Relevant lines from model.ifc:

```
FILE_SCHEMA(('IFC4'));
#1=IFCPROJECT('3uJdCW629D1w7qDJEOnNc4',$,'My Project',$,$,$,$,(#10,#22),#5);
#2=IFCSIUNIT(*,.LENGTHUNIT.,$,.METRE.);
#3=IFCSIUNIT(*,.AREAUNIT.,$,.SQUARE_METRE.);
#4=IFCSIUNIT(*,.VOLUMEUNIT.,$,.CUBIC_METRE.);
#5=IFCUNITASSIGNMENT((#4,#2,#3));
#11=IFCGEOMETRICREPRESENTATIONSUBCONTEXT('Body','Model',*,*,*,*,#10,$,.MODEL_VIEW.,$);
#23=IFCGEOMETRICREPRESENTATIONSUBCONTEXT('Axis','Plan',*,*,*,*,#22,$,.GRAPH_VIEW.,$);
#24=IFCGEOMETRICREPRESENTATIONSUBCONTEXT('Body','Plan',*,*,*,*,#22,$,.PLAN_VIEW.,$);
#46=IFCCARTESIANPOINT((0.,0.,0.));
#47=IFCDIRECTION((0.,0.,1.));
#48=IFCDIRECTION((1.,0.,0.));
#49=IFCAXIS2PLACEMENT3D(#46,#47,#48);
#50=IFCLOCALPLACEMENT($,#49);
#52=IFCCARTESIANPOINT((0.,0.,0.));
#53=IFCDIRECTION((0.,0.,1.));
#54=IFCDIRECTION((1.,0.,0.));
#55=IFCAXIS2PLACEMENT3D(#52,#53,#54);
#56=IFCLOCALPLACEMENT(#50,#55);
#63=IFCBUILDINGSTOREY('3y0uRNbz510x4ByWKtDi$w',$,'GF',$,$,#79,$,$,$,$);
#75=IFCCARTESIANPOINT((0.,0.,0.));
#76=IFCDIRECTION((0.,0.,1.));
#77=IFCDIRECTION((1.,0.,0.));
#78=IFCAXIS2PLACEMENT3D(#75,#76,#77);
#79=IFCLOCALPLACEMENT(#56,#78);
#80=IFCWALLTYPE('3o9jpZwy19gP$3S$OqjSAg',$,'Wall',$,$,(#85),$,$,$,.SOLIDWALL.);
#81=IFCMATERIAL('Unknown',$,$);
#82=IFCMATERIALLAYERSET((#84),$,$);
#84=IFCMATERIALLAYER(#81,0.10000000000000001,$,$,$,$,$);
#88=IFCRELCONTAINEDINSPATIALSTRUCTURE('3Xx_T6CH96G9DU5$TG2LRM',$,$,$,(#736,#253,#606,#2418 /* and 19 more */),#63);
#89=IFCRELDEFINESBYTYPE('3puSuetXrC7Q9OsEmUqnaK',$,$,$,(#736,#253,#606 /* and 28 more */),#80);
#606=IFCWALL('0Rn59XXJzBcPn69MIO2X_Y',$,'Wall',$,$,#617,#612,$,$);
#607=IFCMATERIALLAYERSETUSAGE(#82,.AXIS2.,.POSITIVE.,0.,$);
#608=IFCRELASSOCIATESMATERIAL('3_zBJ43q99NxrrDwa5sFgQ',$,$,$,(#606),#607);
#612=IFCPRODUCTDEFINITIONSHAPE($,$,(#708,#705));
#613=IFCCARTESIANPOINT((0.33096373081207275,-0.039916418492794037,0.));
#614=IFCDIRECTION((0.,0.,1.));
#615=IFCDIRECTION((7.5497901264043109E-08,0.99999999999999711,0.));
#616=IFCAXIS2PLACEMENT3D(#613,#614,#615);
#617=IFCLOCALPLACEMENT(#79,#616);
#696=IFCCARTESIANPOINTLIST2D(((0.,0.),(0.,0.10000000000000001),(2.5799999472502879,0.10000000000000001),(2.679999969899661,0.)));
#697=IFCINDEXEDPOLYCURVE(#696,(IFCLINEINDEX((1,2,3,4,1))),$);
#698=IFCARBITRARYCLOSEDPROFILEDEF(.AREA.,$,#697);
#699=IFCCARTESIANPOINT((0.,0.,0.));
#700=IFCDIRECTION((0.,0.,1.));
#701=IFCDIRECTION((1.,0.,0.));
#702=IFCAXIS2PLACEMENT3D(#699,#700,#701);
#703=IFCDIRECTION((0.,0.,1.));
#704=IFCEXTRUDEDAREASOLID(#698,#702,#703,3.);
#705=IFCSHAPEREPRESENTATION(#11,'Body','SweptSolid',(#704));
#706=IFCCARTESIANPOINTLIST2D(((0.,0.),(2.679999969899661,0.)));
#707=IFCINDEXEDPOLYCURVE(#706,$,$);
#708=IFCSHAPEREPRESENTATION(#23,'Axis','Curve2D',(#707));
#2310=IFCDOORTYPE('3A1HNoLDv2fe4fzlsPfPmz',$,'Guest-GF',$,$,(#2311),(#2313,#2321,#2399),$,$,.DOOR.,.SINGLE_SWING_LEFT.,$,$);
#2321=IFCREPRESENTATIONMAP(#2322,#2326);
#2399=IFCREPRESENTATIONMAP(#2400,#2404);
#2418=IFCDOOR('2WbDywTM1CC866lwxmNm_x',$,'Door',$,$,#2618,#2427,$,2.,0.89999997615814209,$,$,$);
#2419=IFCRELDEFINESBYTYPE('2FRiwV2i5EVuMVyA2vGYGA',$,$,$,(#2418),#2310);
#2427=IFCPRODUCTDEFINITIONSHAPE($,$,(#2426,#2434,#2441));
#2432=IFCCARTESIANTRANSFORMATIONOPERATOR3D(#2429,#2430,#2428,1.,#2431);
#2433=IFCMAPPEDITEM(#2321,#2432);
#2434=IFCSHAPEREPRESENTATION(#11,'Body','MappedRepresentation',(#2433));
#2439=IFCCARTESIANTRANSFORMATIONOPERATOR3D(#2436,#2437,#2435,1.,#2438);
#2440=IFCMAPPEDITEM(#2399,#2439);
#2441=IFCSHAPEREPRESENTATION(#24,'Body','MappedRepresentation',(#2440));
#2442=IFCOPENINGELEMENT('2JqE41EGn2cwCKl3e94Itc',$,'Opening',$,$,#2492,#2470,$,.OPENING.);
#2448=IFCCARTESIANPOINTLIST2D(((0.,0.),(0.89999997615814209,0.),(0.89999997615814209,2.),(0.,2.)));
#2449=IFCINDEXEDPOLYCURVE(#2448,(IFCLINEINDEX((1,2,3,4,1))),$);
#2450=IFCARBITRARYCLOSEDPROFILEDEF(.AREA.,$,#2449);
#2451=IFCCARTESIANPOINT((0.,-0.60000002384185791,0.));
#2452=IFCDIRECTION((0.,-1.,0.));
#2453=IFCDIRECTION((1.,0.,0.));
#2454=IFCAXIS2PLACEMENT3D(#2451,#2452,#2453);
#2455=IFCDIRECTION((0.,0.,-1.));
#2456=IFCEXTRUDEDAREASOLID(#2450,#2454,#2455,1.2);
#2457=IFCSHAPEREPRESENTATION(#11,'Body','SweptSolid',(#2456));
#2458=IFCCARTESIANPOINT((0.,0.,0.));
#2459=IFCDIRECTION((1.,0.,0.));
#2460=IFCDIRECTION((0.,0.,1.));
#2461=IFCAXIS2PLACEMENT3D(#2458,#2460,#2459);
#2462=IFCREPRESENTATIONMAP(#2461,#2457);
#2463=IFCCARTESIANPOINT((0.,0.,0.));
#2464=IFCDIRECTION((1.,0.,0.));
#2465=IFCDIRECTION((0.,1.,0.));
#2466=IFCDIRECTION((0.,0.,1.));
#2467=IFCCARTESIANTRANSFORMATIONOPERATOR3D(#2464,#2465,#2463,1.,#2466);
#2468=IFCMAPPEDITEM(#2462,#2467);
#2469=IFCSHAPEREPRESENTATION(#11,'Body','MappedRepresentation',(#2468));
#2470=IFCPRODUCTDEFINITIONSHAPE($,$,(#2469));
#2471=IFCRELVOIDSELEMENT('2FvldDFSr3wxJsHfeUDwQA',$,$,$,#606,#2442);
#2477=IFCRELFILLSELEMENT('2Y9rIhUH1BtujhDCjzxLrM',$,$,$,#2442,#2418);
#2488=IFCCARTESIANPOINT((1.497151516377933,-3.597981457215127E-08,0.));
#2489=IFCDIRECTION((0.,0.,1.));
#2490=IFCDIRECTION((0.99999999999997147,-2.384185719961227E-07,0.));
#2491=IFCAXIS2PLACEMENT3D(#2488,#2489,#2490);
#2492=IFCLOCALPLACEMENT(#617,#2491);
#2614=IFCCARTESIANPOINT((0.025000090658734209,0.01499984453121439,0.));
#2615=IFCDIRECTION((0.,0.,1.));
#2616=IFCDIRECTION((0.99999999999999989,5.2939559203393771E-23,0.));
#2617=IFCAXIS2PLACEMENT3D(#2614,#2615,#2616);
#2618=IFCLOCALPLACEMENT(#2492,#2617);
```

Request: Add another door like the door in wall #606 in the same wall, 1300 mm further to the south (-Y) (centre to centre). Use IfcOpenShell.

```python
import ifcopenshell
import ifcopenshell.api.feature
import ifcopenshell.api.geometry
import ifcopenshell.api.root
import ifcopenshell.geom
import ifcopenshell.util.element
import ifcopenshell.util.placement
import ifcopenshell.util.shape

model = ifcopenshell.open("model.ifc")
settings = ifcopenshell.geom.settings()


def volume(element):
    """Net volume in cubic metres, openings subtracted."""
    shape = ifcopenshell.geom.create_shape(settings, element)
    return ifcopenshell.util.shape.get_volume(shape.geometry)


door = model.by_guid("2WbDywTM1CC866lwxmNm_x")
opening = door.FillsVoids[0].RelatingOpeningElement
wall = opening.VoidsElements[0].RelatingBuildingElement
before = volume(wall)
shift = ifcopenshell.util.placement.get_local_placement(wall.ObjectPlacement)[:3, 0] * -1.3

# copy_class copies the void relationship, type, container and properties, but no geometry.
new_opening = ifcopenshell.api.root.copy_class(model, product=opening)
new_opening.Representation = ifcopenshell.util.element.copy_deep(
    model, opening.Representation, exclude=["IfcGeometricRepresentationContext", "IfcRepresentationMap"]
)
new_door = ifcopenshell.api.root.copy_class(model, product=door)
new_door.Representation = ifcopenshell.util.element.copy_deep(
    model, door.Representation, exclude=["IfcGeometricRepresentationContext", "IfcRepresentationMap"]
)
ifcopenshell.api.feature.add_filling(model, opening=new_opening, element=new_door)

for old, new in ((opening, new_opening), (door, new_door)):
    matrix = ifcopenshell.util.placement.get_local_placement(old.ObjectPlacement)
    matrix[:3, 3] += shift
    ifcopenshell.api.geometry.edit_object_placement(model, product=new, matrix=matrix, is_si=False)

after = volume(wall)

print(f"wall volume {before:.3f} -> {after:.3f} m3")

model.write("model_updated.ifc")
```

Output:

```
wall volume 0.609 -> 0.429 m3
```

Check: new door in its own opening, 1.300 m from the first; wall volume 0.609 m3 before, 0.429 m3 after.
